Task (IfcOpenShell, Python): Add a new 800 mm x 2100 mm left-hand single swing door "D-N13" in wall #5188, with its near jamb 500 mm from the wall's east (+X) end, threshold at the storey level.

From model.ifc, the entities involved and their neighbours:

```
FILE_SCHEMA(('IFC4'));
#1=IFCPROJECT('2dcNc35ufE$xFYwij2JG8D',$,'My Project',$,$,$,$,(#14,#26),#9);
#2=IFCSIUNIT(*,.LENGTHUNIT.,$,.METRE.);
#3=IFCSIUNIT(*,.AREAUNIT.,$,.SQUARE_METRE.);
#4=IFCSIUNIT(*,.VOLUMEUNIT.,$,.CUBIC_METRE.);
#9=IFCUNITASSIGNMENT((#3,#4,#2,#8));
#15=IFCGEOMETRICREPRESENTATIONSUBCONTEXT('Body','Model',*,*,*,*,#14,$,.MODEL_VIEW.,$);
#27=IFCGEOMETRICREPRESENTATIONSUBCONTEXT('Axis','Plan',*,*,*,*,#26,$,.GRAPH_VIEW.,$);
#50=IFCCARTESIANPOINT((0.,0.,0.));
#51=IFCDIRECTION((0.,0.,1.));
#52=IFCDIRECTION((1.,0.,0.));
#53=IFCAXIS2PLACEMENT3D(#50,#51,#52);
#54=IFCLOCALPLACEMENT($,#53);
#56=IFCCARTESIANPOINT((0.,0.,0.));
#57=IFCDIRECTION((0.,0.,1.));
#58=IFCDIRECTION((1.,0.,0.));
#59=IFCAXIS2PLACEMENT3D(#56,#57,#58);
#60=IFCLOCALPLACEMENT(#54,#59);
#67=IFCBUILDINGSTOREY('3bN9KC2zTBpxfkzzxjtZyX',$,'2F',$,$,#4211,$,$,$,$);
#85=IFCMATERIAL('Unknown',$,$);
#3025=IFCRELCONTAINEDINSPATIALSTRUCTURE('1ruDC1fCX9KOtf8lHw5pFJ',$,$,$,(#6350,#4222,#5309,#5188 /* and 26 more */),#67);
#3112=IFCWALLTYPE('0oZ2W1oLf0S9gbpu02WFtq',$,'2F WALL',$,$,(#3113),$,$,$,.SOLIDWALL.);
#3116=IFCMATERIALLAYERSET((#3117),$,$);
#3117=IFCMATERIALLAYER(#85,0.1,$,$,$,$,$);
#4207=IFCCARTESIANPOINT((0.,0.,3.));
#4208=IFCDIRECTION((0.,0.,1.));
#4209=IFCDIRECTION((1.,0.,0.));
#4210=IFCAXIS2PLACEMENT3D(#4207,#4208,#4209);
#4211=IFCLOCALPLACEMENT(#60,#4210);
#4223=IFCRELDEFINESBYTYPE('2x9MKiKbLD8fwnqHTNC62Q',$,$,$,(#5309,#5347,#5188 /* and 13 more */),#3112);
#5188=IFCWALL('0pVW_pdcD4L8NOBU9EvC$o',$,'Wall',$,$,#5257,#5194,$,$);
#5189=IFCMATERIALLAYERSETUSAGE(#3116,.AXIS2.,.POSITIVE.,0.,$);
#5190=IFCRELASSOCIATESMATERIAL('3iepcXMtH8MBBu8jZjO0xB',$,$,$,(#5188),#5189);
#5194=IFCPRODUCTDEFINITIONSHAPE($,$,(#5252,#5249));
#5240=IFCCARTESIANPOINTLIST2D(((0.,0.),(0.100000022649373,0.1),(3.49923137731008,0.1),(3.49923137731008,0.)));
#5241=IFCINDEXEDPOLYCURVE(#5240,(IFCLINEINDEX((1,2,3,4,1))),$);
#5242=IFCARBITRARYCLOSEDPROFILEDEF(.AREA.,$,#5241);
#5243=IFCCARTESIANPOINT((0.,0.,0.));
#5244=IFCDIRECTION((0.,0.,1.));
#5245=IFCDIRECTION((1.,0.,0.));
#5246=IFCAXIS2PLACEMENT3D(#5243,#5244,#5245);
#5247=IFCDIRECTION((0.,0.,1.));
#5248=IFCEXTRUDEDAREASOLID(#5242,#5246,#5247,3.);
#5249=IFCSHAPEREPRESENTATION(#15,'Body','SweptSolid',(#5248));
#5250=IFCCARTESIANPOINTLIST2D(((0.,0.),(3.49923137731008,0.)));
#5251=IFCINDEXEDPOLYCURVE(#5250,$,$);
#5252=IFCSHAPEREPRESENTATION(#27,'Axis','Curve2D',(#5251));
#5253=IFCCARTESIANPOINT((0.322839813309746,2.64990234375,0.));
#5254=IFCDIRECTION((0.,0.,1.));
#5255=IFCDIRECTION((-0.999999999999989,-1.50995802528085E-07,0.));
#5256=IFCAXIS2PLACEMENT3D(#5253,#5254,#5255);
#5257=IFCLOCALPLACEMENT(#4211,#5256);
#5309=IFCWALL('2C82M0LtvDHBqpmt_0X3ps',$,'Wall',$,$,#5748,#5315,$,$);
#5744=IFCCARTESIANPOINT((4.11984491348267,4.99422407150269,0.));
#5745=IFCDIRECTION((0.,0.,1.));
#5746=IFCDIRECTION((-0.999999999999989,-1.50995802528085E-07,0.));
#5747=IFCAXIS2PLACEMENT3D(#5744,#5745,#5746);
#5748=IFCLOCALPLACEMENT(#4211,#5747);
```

```python
import numpy as np
import ifcopenshell
import ifcopenshell.api.feature
import ifcopenshell.api.geometry
import ifcopenshell.api.root
import ifcopenshell.api.spatial
import ifcopenshell.geom
import ifcopenshell.util.element
import ifcopenshell.util.placement
import ifcopenshell.util.representation
import ifcopenshell.util.shape
import ifcopenshell.util.unit

model = ifcopenshell.open("model.ifc")
unit_scale = ifcopenshell.util.unit.calculate_unit_scale(model)
settings = ifcopenshell.geom.settings()


def volume(element):
    """Net volume in cubic metres, openings subtracted."""
    shape = ifcopenshell.geom.create_shape(settings, element)
    return ifcopenshell.util.shape.get_volume(shape.geometry)


wall = model.by_id(5188)
storey = ifcopenshell.util.element.get_container(wall, ifc_class="IfcBuildingStorey")
context = ifcopenshell.util.representation.get_context(model, "Model", "Body", "MODEL_VIEW")
before = volume(wall)

width, height, from_end, sill = 0.8, 2.1, 0.5, 0.0  # metres

# The wall runs along its own X axis, and the end named is its -X end.
wall_shape = ifcopenshell.geom.create_shape(settings, wall)
x, y, z = ifcopenshell.util.shape.get_vertices(wall_shape.geometry).T
start = x.min() + from_end
face, thickness = float(y.min()), float(y.max() - y.min())
wall_matrix = ifcopenshell.util.placement.get_local_placement(wall.ObjectPlacement)
level = ifcopenshell.util.placement.get_local_placement(storey.ObjectPlacement)[2, 3]


def in_wall(x, y):
    """Placement at x, y metres in the wall's axes, at sill height."""
    matrix = wall_matrix.copy()
    matrix[:, 3] = wall_matrix @ np.array([x / unit_scale, y / unit_scale, 0.0, 1.0])
    matrix[2, 3] = level + sill / unit_scale
    return matrix


# Opening: a box that overshoots both wall faces by 50 mm.
opening = ifcopenshell.api.root.create_entity(model, ifc_class="IfcOpeningElement", predefined_type="OPENING")
box = ifcopenshell.api.geometry.add_wall_representation(
    model, context=context, length=width, height=height, thickness=thickness + 0.1
)
ifcopenshell.api.geometry.assign_representation(model, product=opening, representation=box)
ifcopenshell.api.geometry.edit_object_placement(model, product=opening, matrix=in_wall(start, face - 0.05), is_si=False)
ifcopenshell.api.feature.add_feature(model, feature=opening, element=wall)

door = ifcopenshell.api.root.create_entity(model, ifc_class="IfcDoor", name="D-N13", predefined_type="DOOR")
door.OverallWidth, door.OverallHeight = width / unit_scale, height / unit_scale
door.OperationType = "SINGLE_SWING_LEFT"
body = ifcopenshell.api.geometry.add_door_representation(
    model,
    context=context,
    overall_width=door.OverallWidth,
    overall_height=door.OverallHeight,
    operation_type="SINGLE_SWING_LEFT",
    lining_properties={"LiningDepth": thickness / unit_scale, "ThresholdDepth": thickness / unit_scale},
)
ifcopenshell.api.geometry.assign_representation(model, product=door, representation=body)
ifcopenshell.api.spatial.assign_container(model, products=[door], relating_structure=storey)
ifcopenshell.api.feature.add_filling(model, opening=opening, element=door)

# The lining spans the wall, so the door starts at the wall face.
ifcopenshell.api.geometry.edit_object_placement(model, product=door, matrix=in_wall(start, face), is_si=False)

after = volume(wall)

print(f"wall volume {before:.3f} -> {after:.3f} m3")

model.write("model_updated.ifc")
```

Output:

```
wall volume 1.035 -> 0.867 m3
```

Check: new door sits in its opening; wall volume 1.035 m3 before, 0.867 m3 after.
